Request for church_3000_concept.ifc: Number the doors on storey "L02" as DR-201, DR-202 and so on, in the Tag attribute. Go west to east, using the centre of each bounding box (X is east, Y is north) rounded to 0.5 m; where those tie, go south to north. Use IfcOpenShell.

First a look at what the model holds.

```python
import ifcopenshell
import ifcopenshell.util.element
import ifcopenshell.util.placement

model = ifcopenshell.open("church_3000_concept.ifc")
print(model.schema)
storey = next(s for s in model.by_type("IfcBuildingStorey") if s.Name == "L02")
doors = [e for e in ifcopenshell.util.element.get_decomposition(storey) if e.is_a("IfcDoor")]
for e in sorted(doors, key=lambda e: e.id()):
    origin = ifcopenshell.util.placement.get_local_placement(e.ObjectPlacement)[:3, 3]
    print(e.id(), e.Tag, e.Name, origin.round(2) + 0.0, sep=" | ")
```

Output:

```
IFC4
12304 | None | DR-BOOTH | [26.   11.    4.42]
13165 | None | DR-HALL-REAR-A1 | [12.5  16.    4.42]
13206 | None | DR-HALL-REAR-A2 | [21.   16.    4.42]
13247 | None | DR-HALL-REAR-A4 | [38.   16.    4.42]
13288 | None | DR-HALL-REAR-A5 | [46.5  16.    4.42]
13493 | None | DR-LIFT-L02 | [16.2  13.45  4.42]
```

```python
import ifcopenshell
import ifcopenshell.geom
import ifcopenshell.util.element
import ifcopenshell.util.shape

model = ifcopenshell.open("church_3000_concept.ifc")
settings = ifcopenshell.geom.settings()
settings.set("use-world-coords", True)


def centre(element):
    shape = ifcopenshell.geom.create_shape(settings, element)
    return ifcopenshell.util.shape.get_bbox_centroid(shape.geometry)


storey = next(s for s in model.by_type("IfcBuildingStorey") if s.Name == "L02")
doors = [e for e in ifcopenshell.util.element.get_decomposition(storey) if e.is_a("IfcDoor")]

# Insertion points can sit at a corner or the storey origin, so sort by the geometry (in metres).
centres = {e: centre(e) for e in doors}
doors.sort(key=lambda e: (round(centres[e][0] / 0.5), centres[e][1]))

for i, e in enumerate(doors, start=1):
    number = f"DR-2{i:02d}"
    e.Tag = number
    print(e.id(), number)

model.write("church_3000_concept_updated.ifc")
```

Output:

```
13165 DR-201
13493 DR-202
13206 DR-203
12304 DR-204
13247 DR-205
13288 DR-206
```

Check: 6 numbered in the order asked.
